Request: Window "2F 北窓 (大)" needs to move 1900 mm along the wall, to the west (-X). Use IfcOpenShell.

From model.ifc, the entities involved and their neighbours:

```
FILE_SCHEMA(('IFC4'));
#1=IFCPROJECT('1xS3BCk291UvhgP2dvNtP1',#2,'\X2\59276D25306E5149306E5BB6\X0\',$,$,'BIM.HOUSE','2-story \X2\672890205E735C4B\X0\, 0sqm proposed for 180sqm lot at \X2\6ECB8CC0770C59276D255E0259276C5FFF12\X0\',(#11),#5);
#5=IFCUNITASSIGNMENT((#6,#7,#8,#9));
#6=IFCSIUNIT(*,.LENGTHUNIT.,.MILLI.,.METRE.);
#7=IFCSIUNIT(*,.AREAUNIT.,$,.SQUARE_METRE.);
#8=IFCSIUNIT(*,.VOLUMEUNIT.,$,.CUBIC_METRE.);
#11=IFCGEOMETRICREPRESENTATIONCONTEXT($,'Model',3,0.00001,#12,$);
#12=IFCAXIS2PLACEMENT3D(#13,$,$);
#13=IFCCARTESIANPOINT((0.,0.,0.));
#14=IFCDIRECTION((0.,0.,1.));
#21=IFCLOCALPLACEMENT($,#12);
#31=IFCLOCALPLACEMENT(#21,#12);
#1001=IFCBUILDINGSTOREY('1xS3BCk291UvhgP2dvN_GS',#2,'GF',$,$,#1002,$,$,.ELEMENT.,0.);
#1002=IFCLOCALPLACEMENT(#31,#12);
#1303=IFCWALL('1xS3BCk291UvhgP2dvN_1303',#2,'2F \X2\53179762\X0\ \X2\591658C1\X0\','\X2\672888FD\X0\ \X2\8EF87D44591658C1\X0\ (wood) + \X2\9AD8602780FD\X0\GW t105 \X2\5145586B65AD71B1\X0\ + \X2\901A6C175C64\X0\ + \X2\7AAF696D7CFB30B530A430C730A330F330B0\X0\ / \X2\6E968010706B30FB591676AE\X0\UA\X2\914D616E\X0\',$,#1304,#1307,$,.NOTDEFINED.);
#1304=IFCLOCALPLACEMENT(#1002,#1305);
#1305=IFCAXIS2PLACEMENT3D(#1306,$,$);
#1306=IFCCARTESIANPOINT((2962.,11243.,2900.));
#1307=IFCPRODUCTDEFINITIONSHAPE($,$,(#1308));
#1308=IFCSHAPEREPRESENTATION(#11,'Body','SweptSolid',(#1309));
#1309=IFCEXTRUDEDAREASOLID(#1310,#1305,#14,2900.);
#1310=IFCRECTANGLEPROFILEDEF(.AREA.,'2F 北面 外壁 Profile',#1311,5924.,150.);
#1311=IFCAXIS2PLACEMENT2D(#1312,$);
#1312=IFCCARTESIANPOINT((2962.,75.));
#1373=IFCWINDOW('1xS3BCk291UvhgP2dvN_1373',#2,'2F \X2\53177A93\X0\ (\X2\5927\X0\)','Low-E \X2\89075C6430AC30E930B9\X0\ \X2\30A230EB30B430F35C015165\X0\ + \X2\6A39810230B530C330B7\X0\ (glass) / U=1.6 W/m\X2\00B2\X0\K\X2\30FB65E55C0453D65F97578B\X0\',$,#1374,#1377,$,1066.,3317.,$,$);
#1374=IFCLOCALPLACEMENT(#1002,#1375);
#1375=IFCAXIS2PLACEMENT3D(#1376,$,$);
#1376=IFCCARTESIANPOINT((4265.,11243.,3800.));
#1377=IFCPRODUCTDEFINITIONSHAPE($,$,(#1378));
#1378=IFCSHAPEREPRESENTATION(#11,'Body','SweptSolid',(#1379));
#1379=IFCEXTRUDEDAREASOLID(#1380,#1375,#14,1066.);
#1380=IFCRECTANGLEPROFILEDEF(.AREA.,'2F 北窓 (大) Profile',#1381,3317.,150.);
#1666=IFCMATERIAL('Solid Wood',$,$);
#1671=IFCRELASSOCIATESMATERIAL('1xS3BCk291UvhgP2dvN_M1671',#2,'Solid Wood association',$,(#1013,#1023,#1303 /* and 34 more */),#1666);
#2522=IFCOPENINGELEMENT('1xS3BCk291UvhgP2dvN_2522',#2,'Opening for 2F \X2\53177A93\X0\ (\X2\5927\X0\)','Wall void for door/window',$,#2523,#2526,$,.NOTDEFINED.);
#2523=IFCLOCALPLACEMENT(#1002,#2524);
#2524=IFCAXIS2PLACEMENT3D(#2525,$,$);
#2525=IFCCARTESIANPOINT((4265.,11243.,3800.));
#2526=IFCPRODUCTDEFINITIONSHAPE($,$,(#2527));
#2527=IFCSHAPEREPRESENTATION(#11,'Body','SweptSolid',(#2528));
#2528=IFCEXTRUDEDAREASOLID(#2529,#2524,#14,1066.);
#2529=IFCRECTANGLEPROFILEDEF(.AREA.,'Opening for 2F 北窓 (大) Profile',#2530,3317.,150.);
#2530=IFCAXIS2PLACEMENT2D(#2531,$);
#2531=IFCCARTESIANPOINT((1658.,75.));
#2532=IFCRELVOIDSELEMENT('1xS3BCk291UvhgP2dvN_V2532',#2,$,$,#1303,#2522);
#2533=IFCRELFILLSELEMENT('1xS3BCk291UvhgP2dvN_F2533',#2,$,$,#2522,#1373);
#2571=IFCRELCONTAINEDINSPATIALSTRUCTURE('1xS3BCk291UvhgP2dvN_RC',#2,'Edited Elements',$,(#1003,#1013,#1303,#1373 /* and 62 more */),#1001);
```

```python
import ifcopenshell
import ifcopenshell.api.geometry
import ifcopenshell.util.placement

model = ifcopenshell.open("model.ifc")

window = model.by_id(1373)
opening = window.FillsVoids[0].RelatingOpeningElement
wall = opening.VoidsElements[0].RelatingBuildingElement

wall_matrix = ifcopenshell.util.placement.get_local_placement(wall.ObjectPlacement)
shift = wall_matrix[:3, 0] * -1900.0
before = ifcopenshell.util.placement.get_local_placement(window.ObjectPlacement)[:3, 3].copy()

# The window is not placed relative to its opening, so move both.
for product in (opening, window):
    matrix = ifcopenshell.util.placement.get_local_placement(product.ObjectPlacement)
    matrix[:3, 3] += shift
    ifcopenshell.api.geometry.edit_object_placement(model, product=product, matrix=matrix, is_si=False)

after = ifcopenshell.util.placement.get_local_placement(window.ObjectPlacement)[:3, 3]
print("window moved by", (after - before).round(3) + 0.0)

model.write("model_rev.ifc")
```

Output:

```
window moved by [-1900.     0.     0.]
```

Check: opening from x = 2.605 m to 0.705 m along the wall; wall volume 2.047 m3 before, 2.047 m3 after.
